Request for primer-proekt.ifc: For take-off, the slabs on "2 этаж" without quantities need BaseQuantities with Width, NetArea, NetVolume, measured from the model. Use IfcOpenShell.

First a look at what the model holds.

```python
import ifcopenshell
import ifcopenshell.util.element
import ifcopenshell.util.unit

model = ifcopenshell.open("primer-proekt.ifc")
print(model.schema)
for unit_type in ("LENGTHUNIT", "AREAUNIT", "VOLUMEUNIT"):
    print(unit_type, ifcopenshell.util.unit.calculate_unit_scale(model, unit_type))
storey = next(s for s in model.by_type("IfcBuildingStorey") if s.Name == "2 этаж")
slabs = [e for e in ifcopenshell.util.element.get_decomposition(storey) if e.is_a("IfcSlab")]
for e in sorted(slabs, key=lambda e: e.id()):
    print(e.id(), e.is_a(), e.Name, list(ifcopenshell.util.element.get_psets(e, qtos_only=True)), sep=" | ")
```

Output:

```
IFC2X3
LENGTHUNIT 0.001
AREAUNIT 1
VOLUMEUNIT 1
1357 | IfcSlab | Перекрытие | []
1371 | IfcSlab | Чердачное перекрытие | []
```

```python
import ifcopenshell
import ifcopenshell.api.pset
import ifcopenshell.geom
import ifcopenshell.util.element
import ifcopenshell.util.shape
import ifcopenshell.util.unit

model = ifcopenshell.open("primer-proekt.ifc")
unit_scale = ifcopenshell.util.unit.calculate_unit_scale(model)
area_scale = ifcopenshell.util.unit.calculate_unit_scale(model, "AREAUNIT")
volume_scale = ifcopenshell.util.unit.calculate_unit_scale(model, "VOLUMEUNIT")
settings = ifcopenshell.geom.settings()

storey = next(s for s in model.by_type("IfcBuildingStorey") if s.Name == "2 этаж")
slabs = [e for e in ifcopenshell.util.element.get_decomposition(storey) if e.is_a("IfcSlab")]

for e in sorted(slabs, key=lambda e: e.id()):
    if ifcopenshell.util.element.get_psets(e, qtos_only=True, should_inherit=False):
        continue
    # Geometry comes back in metres, in the element's own axes.
    shape = ifcopenshell.geom.create_shape(settings, e)
    values = {
        "Width": ifcopenshell.util.shape.get_z(shape.geometry) / unit_scale,
        "NetArea": ifcopenshell.util.shape.get_footprint_area(shape.geometry) / area_scale,
        "NetVolume": ifcopenshell.util.shape.get_volume(shape.geometry) / volume_scale,
    }
    qto = ifcopenshell.api.pset.add_qto(model, product=e, name="BaseQuantities")
    ifcopenshell.api.pset.edit_qto(model, qto=qto, properties=values)
    print(e.id(), {k: round(v, 3) for k, v in values.items()})

model.write("primer-proekt_edited.ifc")
```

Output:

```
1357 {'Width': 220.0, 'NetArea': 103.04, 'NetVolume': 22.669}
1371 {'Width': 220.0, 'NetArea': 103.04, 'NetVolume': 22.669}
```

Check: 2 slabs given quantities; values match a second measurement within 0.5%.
